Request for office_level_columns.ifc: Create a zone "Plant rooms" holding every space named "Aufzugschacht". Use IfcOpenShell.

First a look at what the model holds.

```python
import ifcopenshell

model = ifcopenshell.open("office_level_columns.ifc")
print(model.schema)
seen = {}
for space in model.by_type("IfcSpace"):
    seen[space.LongName] = seen.get(space.LongName, 0) + 1
for name, count in sorted(seen.items(), key=str):
    print(count, "x", name)
print("zones:", [z.Name for z in model.by_type("IfcZone")][:20])
```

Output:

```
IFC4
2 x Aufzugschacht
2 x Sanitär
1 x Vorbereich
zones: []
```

```python
import ifcopenshell
import ifcopenshell.api.group
import ifcopenshell.api.root

model = ifcopenshell.open("office_level_columns.ifc")

names = {"Aufzugschacht"}
spaces = [s for s in model.by_type("IfcSpace") if s.LongName in names]

zone = ifcopenshell.api.root.create_entity(model, ifc_class="IfcZone", name="Plant rooms")
ifcopenshell.api.group.assign_group(model, products=spaces, group=zone)
print(len(spaces), "spaces in", zone.Name)

model.write("office_level_columns_edited.ifc")
```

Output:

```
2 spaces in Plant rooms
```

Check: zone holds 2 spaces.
